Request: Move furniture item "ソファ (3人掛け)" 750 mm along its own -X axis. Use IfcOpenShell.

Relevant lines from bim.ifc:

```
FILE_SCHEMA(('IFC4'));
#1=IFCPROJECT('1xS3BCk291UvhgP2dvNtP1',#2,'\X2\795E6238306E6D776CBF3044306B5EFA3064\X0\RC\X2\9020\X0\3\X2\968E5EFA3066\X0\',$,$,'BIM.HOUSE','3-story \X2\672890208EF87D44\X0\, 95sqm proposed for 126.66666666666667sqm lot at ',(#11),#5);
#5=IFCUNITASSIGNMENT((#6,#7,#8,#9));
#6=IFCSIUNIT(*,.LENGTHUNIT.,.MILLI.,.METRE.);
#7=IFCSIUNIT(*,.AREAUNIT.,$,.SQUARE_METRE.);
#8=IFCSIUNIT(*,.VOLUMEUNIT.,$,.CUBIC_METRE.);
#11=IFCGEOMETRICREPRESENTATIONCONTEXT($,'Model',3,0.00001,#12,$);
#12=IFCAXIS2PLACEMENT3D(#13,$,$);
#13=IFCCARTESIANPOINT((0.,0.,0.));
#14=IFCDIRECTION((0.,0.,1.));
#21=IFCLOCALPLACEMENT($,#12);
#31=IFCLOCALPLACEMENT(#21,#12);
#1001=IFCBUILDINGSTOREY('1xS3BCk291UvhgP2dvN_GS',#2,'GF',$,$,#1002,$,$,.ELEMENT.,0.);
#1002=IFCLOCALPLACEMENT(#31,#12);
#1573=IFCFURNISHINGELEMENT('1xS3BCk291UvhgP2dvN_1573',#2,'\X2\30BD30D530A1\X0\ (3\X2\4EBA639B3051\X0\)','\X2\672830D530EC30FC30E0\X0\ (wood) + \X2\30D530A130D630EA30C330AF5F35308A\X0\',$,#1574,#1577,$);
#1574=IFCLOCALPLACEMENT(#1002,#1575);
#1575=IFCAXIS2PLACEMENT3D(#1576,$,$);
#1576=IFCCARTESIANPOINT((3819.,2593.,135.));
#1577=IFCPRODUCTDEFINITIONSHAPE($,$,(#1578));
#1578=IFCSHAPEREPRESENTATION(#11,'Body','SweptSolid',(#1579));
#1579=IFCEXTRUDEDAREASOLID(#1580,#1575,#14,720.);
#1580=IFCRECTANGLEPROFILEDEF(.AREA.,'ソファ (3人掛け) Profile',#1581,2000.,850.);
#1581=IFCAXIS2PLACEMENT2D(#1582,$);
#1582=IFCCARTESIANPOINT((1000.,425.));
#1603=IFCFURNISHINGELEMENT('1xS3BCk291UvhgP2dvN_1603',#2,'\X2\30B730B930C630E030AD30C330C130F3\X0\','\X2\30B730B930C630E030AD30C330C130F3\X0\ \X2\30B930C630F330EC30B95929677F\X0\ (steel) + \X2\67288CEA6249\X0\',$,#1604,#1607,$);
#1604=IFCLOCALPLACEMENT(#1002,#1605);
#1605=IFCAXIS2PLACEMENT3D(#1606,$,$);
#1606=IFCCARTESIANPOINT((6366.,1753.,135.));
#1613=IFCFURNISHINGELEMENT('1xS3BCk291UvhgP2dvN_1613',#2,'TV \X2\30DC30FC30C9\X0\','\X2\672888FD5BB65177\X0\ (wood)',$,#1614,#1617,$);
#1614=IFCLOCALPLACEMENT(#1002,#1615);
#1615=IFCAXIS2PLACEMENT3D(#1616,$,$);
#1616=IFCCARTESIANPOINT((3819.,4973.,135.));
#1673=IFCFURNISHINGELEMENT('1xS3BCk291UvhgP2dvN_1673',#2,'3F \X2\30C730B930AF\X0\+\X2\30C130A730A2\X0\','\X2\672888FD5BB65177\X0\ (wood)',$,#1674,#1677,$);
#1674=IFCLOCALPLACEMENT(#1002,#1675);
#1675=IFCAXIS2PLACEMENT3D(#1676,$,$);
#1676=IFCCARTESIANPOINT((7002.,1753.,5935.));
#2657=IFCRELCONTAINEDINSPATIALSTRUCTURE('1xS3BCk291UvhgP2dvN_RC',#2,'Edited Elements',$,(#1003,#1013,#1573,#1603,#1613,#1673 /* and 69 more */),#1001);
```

```python
import ifcopenshell
import ifcopenshell.api.geometry
import ifcopenshell.util.placement
import ifcopenshell.util.unit

model = ifcopenshell.open("bim.ifc")
unit_scale = ifcopenshell.util.unit.calculate_unit_scale(model)

item = model.by_guid("1xS3BCk291UvhgP2dvN_1573")
matrix = ifcopenshell.util.placement.get_local_placement(item.ObjectPlacement)
matrix[:3, 3] -= matrix[:3, 0] * 0.75 / unit_scale
ifcopenshell.api.geometry.edit_object_placement(model, product=item, matrix=matrix, is_si=False)

print(ifcopenshell.util.placement.get_local_placement(item.ObjectPlacement).round(3) + 0.0)

model.write("bim_edited.ifc")
```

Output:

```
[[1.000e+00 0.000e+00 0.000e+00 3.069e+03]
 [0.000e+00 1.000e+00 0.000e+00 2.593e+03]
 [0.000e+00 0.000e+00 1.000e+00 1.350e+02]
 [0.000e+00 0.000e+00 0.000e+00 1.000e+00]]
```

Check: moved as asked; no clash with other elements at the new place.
